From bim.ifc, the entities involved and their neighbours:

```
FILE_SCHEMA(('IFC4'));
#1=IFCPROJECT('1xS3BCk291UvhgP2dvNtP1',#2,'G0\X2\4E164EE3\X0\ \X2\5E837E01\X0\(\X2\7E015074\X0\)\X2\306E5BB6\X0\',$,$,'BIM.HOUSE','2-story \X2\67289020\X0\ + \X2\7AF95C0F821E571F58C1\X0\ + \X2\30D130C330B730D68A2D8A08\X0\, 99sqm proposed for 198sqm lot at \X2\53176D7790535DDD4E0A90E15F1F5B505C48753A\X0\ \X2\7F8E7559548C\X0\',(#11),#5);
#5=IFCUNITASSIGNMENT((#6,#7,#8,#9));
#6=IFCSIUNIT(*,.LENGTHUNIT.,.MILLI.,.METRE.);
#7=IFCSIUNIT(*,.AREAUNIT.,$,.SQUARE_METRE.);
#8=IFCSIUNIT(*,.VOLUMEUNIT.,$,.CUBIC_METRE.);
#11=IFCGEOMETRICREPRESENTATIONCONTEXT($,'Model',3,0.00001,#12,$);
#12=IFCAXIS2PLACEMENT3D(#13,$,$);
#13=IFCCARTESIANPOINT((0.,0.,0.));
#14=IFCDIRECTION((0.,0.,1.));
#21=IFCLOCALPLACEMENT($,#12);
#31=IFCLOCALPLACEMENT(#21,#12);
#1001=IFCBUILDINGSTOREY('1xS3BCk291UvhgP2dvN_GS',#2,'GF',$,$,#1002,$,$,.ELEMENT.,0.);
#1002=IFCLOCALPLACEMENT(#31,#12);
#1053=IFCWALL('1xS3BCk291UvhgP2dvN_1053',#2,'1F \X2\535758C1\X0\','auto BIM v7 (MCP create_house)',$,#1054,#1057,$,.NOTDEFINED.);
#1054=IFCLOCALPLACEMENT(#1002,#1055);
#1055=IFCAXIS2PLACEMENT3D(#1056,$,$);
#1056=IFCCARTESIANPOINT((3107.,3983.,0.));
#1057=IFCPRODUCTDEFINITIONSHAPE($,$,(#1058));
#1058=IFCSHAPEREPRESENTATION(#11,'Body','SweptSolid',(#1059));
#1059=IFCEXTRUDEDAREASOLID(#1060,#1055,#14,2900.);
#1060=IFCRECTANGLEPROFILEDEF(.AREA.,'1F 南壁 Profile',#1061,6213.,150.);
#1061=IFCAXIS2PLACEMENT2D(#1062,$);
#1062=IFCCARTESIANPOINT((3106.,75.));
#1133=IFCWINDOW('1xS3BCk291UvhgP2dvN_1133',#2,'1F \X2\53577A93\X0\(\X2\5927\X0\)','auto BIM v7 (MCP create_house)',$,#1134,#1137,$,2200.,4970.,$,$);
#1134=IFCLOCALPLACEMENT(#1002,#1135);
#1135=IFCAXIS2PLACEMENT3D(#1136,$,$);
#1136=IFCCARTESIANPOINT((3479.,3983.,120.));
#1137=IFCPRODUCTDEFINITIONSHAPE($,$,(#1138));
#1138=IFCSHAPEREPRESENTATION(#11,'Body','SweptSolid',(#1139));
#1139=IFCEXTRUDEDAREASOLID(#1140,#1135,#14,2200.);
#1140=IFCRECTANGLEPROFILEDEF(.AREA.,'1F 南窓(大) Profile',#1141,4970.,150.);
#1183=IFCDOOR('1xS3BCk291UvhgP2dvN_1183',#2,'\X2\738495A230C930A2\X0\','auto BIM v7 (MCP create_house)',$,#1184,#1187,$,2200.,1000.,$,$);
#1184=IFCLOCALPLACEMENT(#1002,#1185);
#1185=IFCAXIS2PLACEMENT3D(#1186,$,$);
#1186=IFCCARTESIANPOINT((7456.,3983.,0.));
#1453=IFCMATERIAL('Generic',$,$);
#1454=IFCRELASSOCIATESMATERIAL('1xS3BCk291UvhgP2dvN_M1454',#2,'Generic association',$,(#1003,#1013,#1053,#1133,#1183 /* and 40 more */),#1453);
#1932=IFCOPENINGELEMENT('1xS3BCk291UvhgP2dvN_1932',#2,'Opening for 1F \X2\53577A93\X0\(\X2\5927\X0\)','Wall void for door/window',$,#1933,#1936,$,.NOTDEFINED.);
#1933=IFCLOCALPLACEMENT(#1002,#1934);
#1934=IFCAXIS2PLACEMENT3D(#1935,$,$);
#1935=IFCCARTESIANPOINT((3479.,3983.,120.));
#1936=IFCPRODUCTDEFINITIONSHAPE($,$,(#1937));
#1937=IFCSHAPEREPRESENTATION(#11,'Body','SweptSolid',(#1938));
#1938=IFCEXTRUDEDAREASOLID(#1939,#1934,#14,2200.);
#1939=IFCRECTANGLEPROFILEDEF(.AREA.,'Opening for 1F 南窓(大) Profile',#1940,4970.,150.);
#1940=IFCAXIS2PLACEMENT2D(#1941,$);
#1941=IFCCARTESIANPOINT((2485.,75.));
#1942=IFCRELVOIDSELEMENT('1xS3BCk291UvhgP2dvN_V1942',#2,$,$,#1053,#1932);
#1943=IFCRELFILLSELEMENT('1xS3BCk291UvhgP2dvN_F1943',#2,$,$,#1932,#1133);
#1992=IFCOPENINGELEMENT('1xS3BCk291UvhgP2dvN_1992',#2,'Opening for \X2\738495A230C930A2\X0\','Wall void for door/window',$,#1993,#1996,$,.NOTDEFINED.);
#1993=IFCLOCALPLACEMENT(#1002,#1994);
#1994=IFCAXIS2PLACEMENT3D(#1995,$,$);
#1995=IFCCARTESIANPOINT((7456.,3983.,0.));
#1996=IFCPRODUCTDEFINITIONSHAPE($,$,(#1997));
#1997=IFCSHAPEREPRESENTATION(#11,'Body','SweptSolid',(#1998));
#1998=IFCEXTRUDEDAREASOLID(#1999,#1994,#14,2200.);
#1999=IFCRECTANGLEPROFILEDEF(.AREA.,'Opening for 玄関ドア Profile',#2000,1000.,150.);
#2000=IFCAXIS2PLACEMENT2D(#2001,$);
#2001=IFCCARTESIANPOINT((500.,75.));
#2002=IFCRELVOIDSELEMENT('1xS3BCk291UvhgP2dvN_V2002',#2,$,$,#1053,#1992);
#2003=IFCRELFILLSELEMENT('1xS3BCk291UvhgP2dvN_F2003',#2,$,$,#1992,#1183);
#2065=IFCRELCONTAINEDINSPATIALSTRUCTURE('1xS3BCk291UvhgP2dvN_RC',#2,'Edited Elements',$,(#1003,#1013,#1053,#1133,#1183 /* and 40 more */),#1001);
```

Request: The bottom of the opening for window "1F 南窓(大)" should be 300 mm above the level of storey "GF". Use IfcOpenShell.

```python
import numpy as np
import ifcopenshell
import ifcopenshell.api.geometry
import ifcopenshell.geom
import ifcopenshell.util.element
import ifcopenshell.util.placement
import ifcopenshell.util.shape
import ifcopenshell.util.unit

model = ifcopenshell.open("bim.ifc")
unit_scale = ifcopenshell.util.unit.calculate_unit_scale(model)

window = model.by_guid("1xS3BCk291UvhgP2dvN_1133")
opening = window.FillsVoids[0].RelatingOpeningElement
storey = ifcopenshell.util.element.get_container(window, ifc_class="IfcBuildingStorey")
level = ifcopenshell.util.placement.get_local_placement(storey.ObjectPlacement)[2, 3]

# The opening's origin need not be at the sill, so measure its lowest point.
shape = ifcopenshell.geom.create_shape(ifcopenshell.geom.settings(), opening)
bottom = ifcopenshell.util.shape.get_shape_bottom_elevation(shape, shape.geometry) / unit_scale
dz = level + 0.3 / unit_scale - bottom

shift = np.array([0.0, 0.0, dz])
# The window is not placed relative to its opening, so move both.
for product in (opening, window):
    matrix = ifcopenshell.util.placement.get_local_placement(product.ObjectPlacement)
    matrix[:3, 3] += shift
    ifcopenshell.api.geometry.edit_object_placement(model, product=product, matrix=matrix, is_si=False)

print(f"moved by {dz * unit_scale:+.3f} m")

model.write("bim_edited.ifc")
```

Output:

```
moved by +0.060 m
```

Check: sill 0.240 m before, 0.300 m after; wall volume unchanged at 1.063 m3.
